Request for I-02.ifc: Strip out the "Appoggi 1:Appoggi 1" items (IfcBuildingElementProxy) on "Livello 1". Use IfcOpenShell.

First a look at what the model holds.

```python
import ifcopenshell
import ifcopenshell.util.element

model = ifcopenshell.open("I-02.ifc")
print(model.schema)
storey = next(s for s in model.by_type("IfcBuildingStorey") if s.Name == "Livello 1")
proxies = [e for e in ifcopenshell.util.element.get_decomposition(storey) if e.is_a("IfcBuildingElementProxy")]
seen = {}
for e in proxies:
    element_type = ifcopenshell.util.element.get_type(e)
    name = element_type.Name if element_type not in (None, e) else None
    seen[name] = seen.get(name, 0) + 1
for name, count in sorted(seen.items(), key=str):
    print(count, "x", name)
```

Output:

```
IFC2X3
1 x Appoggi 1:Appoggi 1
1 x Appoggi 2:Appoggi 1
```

```python
import ifcopenshell
import ifcopenshell.api.root
import ifcopenshell.util.element

model = ifcopenshell.open("I-02.ifc")

storey = next(s for s in model.by_type("IfcBuildingStorey") if s.Name == "Livello 1")
proxies = [e for e in ifcopenshell.util.element.get_decomposition(storey) if e.is_a("IfcBuildingElementProxy")]
targets = [e for e in proxies if (t := ifcopenshell.util.element.get_type(e)) not in (None, e) and t.Name == "Appoggi 1:Appoggi 1"]

for e in targets:
    ifcopenshell.api.root.remove_product(model, product=e)
print(len(targets), "removed")

model.write("I-02_updated.ifc")
```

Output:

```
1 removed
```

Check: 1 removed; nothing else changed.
